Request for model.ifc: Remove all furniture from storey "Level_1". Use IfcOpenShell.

First a look at what the model holds.

```python
import ifcopenshell
import ifcopenshell.util.element

model = ifcopenshell.open("model.ifc")
print(model.schema)
storey = next(s for s in model.by_type("IfcBuildingStorey") if s.Name == "Level_1")
furniture = [e for e in ifcopenshell.util.element.get_decomposition(storey) if e.is_a("IfcFurnishingElement")]
seen = {}
for e in furniture:
    element_type = ifcopenshell.util.element.get_type(e)
    name = element_type.Name if element_type not in (None, e) else None
    seen[name] = seen.get(name, 0) + 1
for name, count in sorted(seen.items(), key=str):
    print(count, "x", name)
```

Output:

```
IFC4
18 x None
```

```python
import ifcopenshell
import ifcopenshell.api.root
import ifcopenshell.util.element

model = ifcopenshell.open("model.ifc")

storey = next(s for s in model.by_type("IfcBuildingStorey") if s.Name == "Level_1")
furniture = [e for e in ifcopenshell.util.element.get_decomposition(storey) if e.is_a("IfcFurnishingElement")]

for e in furniture:
    ifcopenshell.api.root.remove_product(model, product=e)
print(len(furniture), "removed")

model.write("model_rev.ifc")
```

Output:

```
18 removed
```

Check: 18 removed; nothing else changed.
